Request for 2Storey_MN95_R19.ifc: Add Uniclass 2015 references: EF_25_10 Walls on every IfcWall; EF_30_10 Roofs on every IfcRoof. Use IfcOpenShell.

First a look at what the model holds.

```python
import ifcopenshell

model = ifcopenshell.open("2Storey_MN95_R19.ifc")
print(model.schema)
print("classifications:", [c.Name for c in model.by_type("IfcClassification")])
for ifc_class in ("IfcDoor", "IfcRoof", "IfcStair", "IfcWall", "IfcWindow"):
    print(ifc_class, len(model.by_type(ifc_class)))
```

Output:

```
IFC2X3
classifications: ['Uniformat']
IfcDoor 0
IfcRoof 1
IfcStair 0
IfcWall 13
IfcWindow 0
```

```python
import ifcopenshell
import ifcopenshell.api.classification

model = ifcopenshell.open("2Storey_MN95_R19.ifc")

# IFC2X3 requires Source and Edition and has no link from the project to the system.
system = model.create_entity("IfcClassification", Source="NBS", Edition="2015", Name="Uniclass 2015")

codes = {
    "IfcWall": ("EF_25_10", "Walls"),
    "IfcRoof": ("EF_30_10", "Roofs"),
}
for ifc_class, (code, name) in codes.items():
    products = model.by_type(ifc_class)
    ifcopenshell.api.classification.add_reference(
        model, products=products, classification=system, identification=code, name=name
    )
    print(code, len(products))

model.write("2Storey_MN95_R19_edited.ifc")
```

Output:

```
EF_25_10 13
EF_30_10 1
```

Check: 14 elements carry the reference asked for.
